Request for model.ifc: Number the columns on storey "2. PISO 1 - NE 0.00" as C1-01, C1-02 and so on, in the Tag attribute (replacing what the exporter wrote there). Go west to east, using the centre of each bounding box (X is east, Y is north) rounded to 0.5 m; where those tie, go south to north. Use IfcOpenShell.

First a look at what the model holds.

```python
import ifcopenshell
import ifcopenshell.util.element
import ifcopenshell.util.placement

model = ifcopenshell.open("model.ifc")
print(model.schema)
storey = next(s for s in model.by_type("IfcBuildingStorey") if s.Name == "2. PISO 1 - NE 0.00")
columns = [e for e in ifcopenshell.util.element.get_decomposition(storey) if e.is_a("IfcColumn")]
for e in sorted(columns, key=lambda e: e.id()):
    origin = ifcopenshell.util.placement.get_local_placement(e.ObjectPlacement)[:3, 3]
    print(e.id(), e.Tag, e.Name, origin.round(2) + 0.0, sep=" | ")
```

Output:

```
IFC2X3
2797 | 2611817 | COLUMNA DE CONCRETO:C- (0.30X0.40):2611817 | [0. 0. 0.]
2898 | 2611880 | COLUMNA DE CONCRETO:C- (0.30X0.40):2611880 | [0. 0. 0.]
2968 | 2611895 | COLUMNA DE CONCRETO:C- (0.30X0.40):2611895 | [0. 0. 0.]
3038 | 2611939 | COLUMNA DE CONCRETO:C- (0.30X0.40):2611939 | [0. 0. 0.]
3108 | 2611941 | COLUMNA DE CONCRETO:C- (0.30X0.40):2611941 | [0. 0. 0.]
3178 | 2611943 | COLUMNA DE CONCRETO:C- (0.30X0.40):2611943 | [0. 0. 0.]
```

```python
import ifcopenshell
import ifcopenshell.geom
import ifcopenshell.util.element
import ifcopenshell.util.shape

model = ifcopenshell.open("model.ifc")
settings = ifcopenshell.geom.settings()
settings.set("use-world-coords", True)


def centre(element):
    shape = ifcopenshell.geom.create_shape(settings, element)
    return ifcopenshell.util.shape.get_bbox_centroid(shape.geometry)


storey = next(s for s in model.by_type("IfcBuildingStorey") if s.Name == "2. PISO 1 - NE 0.00")
columns = [e for e in ifcopenshell.util.element.get_decomposition(storey) if e.is_a("IfcColumn")]

# Insertion points can sit at a corner or the storey origin, so sort by the geometry (in metres).
centres = {e: centre(e) for e in columns}
columns.sort(key=lambda e: (round(centres[e][0] / 0.5), centres[e][1]))

for i, e in enumerate(columns, start=1):
    number = f"C1-{i:02d}"
    e.Tag = number
    print(e.id(), number)

model.write("model_edited.ifc")
```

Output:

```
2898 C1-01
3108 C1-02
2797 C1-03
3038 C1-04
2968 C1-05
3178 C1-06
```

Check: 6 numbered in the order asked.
